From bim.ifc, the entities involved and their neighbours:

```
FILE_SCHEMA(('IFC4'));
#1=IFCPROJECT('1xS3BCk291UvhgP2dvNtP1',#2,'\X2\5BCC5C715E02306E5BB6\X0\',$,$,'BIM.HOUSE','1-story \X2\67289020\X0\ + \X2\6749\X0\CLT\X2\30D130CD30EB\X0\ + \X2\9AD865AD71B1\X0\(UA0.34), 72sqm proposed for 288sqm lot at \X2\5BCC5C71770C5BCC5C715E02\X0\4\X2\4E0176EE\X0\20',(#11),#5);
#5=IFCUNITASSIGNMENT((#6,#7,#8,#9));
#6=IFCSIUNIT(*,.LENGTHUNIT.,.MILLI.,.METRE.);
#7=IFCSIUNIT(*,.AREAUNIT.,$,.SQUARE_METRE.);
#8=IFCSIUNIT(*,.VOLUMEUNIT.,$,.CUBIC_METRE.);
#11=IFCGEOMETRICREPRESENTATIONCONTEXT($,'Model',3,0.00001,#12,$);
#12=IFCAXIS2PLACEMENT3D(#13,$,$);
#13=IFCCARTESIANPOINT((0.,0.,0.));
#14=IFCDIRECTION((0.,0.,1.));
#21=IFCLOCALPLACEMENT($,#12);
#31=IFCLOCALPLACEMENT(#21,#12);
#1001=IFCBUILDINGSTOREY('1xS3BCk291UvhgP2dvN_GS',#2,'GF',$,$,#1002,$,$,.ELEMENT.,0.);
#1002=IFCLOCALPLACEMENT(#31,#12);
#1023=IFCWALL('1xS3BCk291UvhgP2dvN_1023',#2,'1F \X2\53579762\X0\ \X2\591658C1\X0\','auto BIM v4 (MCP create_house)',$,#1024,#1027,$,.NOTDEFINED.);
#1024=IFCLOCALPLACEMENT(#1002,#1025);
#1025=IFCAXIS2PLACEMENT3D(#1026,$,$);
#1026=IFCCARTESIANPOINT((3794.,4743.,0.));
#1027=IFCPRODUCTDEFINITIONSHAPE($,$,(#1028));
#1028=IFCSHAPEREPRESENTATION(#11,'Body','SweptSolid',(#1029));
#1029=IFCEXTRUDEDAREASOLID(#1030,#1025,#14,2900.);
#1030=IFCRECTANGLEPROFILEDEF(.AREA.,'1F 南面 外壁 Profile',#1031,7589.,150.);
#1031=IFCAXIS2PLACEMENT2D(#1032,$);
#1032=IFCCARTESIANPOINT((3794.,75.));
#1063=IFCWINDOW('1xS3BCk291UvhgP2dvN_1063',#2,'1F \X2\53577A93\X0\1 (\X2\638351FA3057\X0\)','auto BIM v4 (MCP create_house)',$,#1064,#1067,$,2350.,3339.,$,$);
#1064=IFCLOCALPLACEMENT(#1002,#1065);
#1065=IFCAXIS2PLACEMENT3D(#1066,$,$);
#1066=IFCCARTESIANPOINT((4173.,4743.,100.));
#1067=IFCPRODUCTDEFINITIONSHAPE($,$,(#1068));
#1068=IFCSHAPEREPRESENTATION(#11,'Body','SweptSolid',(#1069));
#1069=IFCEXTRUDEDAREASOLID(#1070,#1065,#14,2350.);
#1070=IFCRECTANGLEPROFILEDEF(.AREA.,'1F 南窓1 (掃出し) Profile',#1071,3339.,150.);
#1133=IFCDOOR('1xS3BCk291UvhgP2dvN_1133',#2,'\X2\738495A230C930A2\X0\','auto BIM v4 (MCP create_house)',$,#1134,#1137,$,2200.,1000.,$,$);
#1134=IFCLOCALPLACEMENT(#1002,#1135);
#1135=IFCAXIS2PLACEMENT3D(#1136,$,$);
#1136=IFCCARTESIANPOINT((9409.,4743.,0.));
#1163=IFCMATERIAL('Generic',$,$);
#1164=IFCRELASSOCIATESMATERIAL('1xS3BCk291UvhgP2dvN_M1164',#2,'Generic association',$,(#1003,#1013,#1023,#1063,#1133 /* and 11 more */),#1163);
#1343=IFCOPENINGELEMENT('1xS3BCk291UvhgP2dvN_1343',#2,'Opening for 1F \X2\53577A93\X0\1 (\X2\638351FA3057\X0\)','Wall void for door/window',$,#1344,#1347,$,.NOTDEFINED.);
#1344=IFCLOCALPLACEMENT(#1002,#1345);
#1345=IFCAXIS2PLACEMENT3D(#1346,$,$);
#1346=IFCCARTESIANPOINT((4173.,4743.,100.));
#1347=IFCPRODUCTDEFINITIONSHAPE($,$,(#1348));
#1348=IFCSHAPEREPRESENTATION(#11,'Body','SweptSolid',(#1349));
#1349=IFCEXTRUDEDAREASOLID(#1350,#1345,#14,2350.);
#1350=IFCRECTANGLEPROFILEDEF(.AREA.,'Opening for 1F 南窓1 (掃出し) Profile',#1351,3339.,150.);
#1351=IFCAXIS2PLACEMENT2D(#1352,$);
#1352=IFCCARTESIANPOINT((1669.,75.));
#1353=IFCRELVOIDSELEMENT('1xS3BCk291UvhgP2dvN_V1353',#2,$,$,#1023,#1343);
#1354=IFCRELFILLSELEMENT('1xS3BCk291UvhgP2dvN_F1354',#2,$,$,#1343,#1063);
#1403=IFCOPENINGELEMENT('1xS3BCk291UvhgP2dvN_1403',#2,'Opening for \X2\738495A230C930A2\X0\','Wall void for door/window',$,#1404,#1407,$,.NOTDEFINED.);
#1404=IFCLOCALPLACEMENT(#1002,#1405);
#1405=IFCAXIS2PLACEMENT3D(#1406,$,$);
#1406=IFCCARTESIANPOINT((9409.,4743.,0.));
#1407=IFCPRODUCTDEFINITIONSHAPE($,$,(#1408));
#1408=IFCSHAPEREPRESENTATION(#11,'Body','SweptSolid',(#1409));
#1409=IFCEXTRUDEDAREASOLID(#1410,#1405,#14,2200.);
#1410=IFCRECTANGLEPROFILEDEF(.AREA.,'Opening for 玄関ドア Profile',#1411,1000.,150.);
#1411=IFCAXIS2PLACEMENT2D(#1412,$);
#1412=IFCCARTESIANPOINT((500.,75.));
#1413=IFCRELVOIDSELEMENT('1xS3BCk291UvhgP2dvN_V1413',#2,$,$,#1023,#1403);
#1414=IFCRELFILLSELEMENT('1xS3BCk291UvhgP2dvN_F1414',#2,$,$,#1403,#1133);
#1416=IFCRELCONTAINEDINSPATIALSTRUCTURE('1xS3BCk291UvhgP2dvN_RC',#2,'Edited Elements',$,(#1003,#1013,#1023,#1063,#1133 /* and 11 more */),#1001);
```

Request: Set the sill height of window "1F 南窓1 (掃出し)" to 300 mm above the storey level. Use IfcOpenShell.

```python
import numpy as np
import ifcopenshell
import ifcopenshell.api.geometry
import ifcopenshell.geom
import ifcopenshell.util.element
import ifcopenshell.util.placement
import ifcopenshell.util.shape
import ifcopenshell.util.unit

model = ifcopenshell.open("bim.ifc")
unit_scale = ifcopenshell.util.unit.calculate_unit_scale(model)

window = model.by_id(1063)
opening = window.FillsVoids[0].RelatingOpeningElement
storey = ifcopenshell.util.element.get_container(window, ifc_class="IfcBuildingStorey")
level = ifcopenshell.util.placement.get_local_placement(storey.ObjectPlacement)[2, 3]

# The opening's origin need not be at the sill, so measure its lowest point.
shape = ifcopenshell.geom.create_shape(ifcopenshell.geom.settings(), opening)
bottom = ifcopenshell.util.shape.get_shape_bottom_elevation(shape, shape.geometry) / unit_scale
dz = level + 300.0 - bottom

shift = np.array([0.0, 0.0, dz])
# The window is not placed relative to its opening, so move both.
for product in (opening, window):
    matrix = ifcopenshell.util.placement.get_local_placement(product.ObjectPlacement)
    matrix[:3, 3] += shift
    ifcopenshell.api.geometry.edit_object_placement(model, product=product, matrix=matrix, is_si=False)

print(f"moved by {dz * unit_scale:+.3f} m")

model.write("bim_edited.ifc")
```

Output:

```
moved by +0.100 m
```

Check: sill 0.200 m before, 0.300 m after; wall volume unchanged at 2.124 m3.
